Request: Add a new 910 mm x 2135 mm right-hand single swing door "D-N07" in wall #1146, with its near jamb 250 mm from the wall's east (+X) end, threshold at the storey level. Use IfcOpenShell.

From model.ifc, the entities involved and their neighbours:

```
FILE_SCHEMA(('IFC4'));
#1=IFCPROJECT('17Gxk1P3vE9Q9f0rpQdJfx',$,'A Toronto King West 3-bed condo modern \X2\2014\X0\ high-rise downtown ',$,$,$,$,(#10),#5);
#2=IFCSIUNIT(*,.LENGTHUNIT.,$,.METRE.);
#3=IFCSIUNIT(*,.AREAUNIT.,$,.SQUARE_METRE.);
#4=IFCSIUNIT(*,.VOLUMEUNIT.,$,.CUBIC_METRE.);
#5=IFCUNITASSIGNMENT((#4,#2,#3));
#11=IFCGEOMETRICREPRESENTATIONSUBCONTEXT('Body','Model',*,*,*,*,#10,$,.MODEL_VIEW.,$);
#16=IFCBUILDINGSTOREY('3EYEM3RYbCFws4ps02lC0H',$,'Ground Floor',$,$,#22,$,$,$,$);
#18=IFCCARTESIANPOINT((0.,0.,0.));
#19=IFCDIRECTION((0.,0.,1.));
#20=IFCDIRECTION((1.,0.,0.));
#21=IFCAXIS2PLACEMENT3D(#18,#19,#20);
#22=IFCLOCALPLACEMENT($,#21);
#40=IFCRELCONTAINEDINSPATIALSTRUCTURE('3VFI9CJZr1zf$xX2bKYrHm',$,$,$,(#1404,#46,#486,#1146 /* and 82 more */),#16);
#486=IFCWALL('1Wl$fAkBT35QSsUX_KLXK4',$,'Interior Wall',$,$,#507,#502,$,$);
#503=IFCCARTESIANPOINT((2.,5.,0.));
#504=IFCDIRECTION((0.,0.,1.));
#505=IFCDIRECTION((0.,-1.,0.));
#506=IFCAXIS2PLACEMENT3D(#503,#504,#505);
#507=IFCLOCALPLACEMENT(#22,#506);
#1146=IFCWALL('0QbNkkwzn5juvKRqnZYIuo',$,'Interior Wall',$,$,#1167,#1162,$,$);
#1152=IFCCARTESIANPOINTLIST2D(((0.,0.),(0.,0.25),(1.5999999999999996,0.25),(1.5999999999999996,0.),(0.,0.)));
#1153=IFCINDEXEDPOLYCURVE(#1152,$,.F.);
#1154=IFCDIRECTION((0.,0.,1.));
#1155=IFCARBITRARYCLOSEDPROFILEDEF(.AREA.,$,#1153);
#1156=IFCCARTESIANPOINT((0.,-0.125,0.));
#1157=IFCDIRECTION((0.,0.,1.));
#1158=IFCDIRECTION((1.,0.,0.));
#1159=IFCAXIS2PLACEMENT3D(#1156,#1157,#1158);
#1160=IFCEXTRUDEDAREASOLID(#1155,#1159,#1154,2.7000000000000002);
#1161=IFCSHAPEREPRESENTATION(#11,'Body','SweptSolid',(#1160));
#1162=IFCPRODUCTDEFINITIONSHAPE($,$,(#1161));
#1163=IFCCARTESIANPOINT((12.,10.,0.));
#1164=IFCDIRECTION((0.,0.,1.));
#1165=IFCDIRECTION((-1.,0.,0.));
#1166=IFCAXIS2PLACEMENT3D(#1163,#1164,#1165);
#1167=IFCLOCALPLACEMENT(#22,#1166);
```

```python
import numpy as np
import ifcopenshell
import ifcopenshell.api.feature
import ifcopenshell.api.geometry
import ifcopenshell.api.root
import ifcopenshell.api.spatial
import ifcopenshell.geom
import ifcopenshell.util.element
import ifcopenshell.util.placement
import ifcopenshell.util.representation
import ifcopenshell.util.shape
import ifcopenshell.util.unit

model = ifcopenshell.open("model.ifc")
unit_scale = ifcopenshell.util.unit.calculate_unit_scale(model)
settings = ifcopenshell.geom.settings()


def volume(element):
    """Net volume in cubic metres, openings subtracted."""
    shape = ifcopenshell.geom.create_shape(settings, element)
    return ifcopenshell.util.shape.get_volume(shape.geometry)


wall = model.by_guid("0QbNkkwzn5juvKRqnZYIuo")
storey = ifcopenshell.util.element.get_container(wall, ifc_class="IfcBuildingStorey")
context = ifcopenshell.util.representation.get_context(model, "Model", "Body", "MODEL_VIEW")
before = volume(wall)

width, height, from_end, sill = 0.91, 2.135, 0.25, 0.0  # metres

# The wall runs along its own X axis, and the end named is its -X end.
wall_shape = ifcopenshell.geom.create_shape(settings, wall)
x, y, z = ifcopenshell.util.shape.get_vertices(wall_shape.geometry).T
start = x.min() + from_end
face, thickness = float(y.min()), float(y.max() - y.min())
wall_matrix = ifcopenshell.util.placement.get_local_placement(wall.ObjectPlacement)
level = ifcopenshell.util.placement.get_local_placement(storey.ObjectPlacement)[2, 3]


def in_wall(x, y):
    """Placement at x, y metres in the wall's axes, at sill height."""
    matrix = wall_matrix.copy()
    matrix[:, 3] = wall_matrix @ np.array([x / unit_scale, y / unit_scale, 0.0, 1.0])
    matrix[2, 3] = level + sill / unit_scale
    return matrix


# Opening: a box that overshoots both wall faces by 50 mm.
opening = ifcopenshell.api.root.create_entity(model, ifc_class="IfcOpeningElement", predefined_type="OPENING")
box = ifcopenshell.api.geometry.add_wall_representation(
    model, context=context, length=width, height=height, thickness=thickness + 0.1
)
ifcopenshell.api.geometry.assign_representation(model, product=opening, representation=box)
ifcopenshell.api.geometry.edit_object_placement(model, product=opening, matrix=in_wall(start, face - 0.05), is_si=False)
ifcopenshell.api.feature.add_feature(model, feature=opening, element=wall)

door = ifcopenshell.api.root.create_entity(model, ifc_class="IfcDoor", name="D-N07", predefined_type="DOOR")
door.OverallWidth, door.OverallHeight = width / unit_scale, height / unit_scale
door.OperationType = "SINGLE_SWING_RIGHT"
body = ifcopenshell.api.geometry.add_door_representation(
    model,
    context=context,
    overall_width=door.OverallWidth,
    overall_height=door.OverallHeight,
    operation_type="SINGLE_SWING_RIGHT",
    lining_properties={"LiningDepth": thickness / unit_scale, "ThresholdDepth": thickness / unit_scale},
)
ifcopenshell.api.geometry.assign_representation(model, product=door, representation=body)
ifcopenshell.api.spatial.assign_container(model, products=[door], relating_structure=storey)
ifcopenshell.api.feature.add_filling(model, opening=opening, element=door)

# The lining spans the wall, so the door starts at the wall face.
ifcopenshell.api.geometry.edit_object_placement(model, product=door, matrix=in_wall(start, face), is_si=False)

after = volume(wall)

print(f"wall volume {before:.3f} -> {after:.3f} m3")

model.write("model_edited.ifc")
```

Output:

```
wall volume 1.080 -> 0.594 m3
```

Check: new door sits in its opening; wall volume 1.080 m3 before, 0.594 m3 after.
